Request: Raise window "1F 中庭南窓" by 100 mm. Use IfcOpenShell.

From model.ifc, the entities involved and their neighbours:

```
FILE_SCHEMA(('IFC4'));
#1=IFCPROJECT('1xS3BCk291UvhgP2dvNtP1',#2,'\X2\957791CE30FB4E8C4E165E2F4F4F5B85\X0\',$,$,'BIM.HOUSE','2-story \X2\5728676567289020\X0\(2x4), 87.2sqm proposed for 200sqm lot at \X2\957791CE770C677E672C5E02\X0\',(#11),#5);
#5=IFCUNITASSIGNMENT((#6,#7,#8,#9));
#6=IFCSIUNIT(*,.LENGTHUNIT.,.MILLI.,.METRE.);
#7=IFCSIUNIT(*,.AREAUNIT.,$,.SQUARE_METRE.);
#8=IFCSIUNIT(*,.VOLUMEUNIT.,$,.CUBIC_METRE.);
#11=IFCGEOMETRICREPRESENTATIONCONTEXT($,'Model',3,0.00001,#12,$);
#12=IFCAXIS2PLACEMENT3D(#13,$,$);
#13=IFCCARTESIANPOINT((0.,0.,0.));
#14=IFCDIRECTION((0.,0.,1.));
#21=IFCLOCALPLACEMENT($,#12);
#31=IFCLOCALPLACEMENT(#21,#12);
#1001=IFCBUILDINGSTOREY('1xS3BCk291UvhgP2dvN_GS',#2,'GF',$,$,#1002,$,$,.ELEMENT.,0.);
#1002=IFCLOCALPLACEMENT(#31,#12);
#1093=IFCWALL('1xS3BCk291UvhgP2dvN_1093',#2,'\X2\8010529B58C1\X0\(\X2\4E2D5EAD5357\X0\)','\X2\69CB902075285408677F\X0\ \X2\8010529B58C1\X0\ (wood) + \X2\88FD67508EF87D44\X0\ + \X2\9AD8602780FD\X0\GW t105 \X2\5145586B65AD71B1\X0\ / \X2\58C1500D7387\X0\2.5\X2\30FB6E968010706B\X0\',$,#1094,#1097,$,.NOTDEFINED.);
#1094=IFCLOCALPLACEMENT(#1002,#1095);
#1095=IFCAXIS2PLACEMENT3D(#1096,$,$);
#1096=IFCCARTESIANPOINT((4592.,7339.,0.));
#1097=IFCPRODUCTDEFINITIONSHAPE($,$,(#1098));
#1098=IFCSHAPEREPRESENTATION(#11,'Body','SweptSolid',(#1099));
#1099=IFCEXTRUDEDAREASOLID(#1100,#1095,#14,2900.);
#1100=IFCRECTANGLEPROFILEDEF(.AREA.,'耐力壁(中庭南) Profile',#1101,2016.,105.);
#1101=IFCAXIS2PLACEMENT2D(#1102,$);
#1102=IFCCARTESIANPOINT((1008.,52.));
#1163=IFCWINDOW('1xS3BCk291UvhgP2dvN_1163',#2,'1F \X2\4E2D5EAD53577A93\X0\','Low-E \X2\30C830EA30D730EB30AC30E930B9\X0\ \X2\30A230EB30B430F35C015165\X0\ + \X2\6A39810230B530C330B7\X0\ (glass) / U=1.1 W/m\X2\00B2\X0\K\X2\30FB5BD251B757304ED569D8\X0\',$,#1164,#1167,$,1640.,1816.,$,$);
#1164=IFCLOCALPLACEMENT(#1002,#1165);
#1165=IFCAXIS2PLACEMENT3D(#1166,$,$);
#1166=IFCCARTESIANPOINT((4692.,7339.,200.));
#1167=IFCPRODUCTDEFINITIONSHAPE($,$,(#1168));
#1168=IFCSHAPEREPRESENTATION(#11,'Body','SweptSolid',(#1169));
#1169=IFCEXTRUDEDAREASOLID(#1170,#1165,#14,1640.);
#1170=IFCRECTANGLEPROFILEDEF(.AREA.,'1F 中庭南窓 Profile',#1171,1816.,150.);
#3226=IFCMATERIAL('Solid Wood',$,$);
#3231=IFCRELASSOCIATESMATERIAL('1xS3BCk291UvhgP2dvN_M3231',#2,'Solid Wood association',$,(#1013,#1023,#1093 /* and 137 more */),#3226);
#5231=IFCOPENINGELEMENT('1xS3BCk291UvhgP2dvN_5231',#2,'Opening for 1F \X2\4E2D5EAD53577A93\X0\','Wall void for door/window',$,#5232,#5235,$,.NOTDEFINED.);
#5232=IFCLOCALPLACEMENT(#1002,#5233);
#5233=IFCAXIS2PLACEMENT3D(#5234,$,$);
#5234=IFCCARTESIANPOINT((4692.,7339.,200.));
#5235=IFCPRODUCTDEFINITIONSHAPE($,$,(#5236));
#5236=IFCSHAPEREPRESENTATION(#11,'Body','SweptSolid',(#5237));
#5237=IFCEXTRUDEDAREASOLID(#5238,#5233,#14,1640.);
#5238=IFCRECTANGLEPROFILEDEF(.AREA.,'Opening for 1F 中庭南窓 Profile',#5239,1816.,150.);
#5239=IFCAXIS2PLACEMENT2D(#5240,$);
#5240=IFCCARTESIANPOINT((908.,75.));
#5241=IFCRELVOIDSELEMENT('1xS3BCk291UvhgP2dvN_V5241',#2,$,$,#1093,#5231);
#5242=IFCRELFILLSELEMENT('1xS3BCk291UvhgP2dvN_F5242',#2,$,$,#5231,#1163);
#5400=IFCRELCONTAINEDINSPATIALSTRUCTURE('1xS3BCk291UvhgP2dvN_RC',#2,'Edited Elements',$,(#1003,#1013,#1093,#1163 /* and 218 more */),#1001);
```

```python
import numpy as np
import ifcopenshell
import ifcopenshell.api.geometry
import ifcopenshell.util.placement
import ifcopenshell.util.unit

model = ifcopenshell.open("model.ifc")
unit_scale = ifcopenshell.util.unit.calculate_unit_scale(model)

window = model.by_guid("1xS3BCk291UvhgP2dvN_1163")
opening = window.FillsVoids[0].RelatingOpeningElement
dz = 0.1 / unit_scale

shift = np.array([0.0, 0.0, dz])
# The window is not placed relative to its opening, so move both.
for product in (opening, window):
    matrix = ifcopenshell.util.placement.get_local_placement(product.ObjectPlacement)
    matrix[:3, 3] += shift
    ifcopenshell.api.geometry.edit_object_placement(model, product=product, matrix=matrix, is_si=False)

print(f"moved by {dz * unit_scale:+.3f} m")

model.write("model_v2.ifc")
```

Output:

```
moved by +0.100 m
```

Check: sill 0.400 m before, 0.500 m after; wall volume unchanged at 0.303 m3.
